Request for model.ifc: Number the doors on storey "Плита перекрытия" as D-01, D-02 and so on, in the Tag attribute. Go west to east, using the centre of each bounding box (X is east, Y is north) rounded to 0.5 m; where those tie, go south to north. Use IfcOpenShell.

First a look at what the model holds.

```python
import ifcopenshell
import ifcopenshell.util.element
import ifcopenshell.util.placement

model = ifcopenshell.open("model.ifc")
print(model.schema)
storey = next(s for s in model.by_type("IfcBuildingStorey") if s.Name == "Плита перекрытия")
doors = [e for e in ifcopenshell.util.element.get_decomposition(storey) if e.is_a("IfcDoor")]
for e in sorted(doors, key=lambda e: e.id()):
    origin = ifcopenshell.util.placement.get_local_placement(e.ObjectPlacement)[:3, 3]
    print(e.id(), e.Tag, e.Name, origin.round(2) + 0.0, sep=" | ")
```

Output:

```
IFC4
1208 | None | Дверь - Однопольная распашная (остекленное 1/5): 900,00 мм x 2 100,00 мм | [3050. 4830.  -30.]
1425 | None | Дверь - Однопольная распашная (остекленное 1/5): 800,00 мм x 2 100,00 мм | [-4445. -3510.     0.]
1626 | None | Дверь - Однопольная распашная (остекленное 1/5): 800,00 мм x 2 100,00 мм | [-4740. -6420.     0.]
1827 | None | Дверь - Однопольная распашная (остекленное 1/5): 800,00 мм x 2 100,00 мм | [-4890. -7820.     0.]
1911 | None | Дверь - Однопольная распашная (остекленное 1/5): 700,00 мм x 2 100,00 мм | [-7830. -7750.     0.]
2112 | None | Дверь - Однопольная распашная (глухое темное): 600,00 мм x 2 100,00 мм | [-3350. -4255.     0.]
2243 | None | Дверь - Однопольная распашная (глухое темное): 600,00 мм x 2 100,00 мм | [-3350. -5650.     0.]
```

```python
import ifcopenshell
import ifcopenshell.geom
import ifcopenshell.util.element
import ifcopenshell.util.shape

model = ifcopenshell.open("model.ifc")
settings = ifcopenshell.geom.settings()
settings.set("use-world-coords", True)


def centre(element):
    shape = ifcopenshell.geom.create_shape(settings, element)
    return ifcopenshell.util.shape.get_bbox_centroid(shape.geometry)


storey = next(s for s in model.by_type("IfcBuildingStorey") if s.Name == "Плита перекрытия")
doors = [e for e in ifcopenshell.util.element.get_decomposition(storey) if e.is_a("IfcDoor")]

# Insertion points can sit at a corner or the storey origin, so sort by the geometry (in metres).
centres = {e: centre(e) for e in doors}
doors.sort(key=lambda e: (round(centres[e][0] / 0.5), centres[e][1]))

for i, e in enumerate(doors, start=1):
    number = f"D-{i:02d}"
    e.Tag = number
    print(e.id(), number)

model.write("model-out.ifc")
```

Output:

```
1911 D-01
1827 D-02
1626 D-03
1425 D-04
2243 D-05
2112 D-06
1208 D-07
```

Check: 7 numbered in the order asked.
